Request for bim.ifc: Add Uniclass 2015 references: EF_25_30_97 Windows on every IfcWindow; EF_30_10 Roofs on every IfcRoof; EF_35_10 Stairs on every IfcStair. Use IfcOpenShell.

First a look at what the model holds.

```python
import ifcopenshell

model = ifcopenshell.open("bim.ifc")
print(model.schema)
print("classifications:", [c.Name for c in model.by_type("IfcClassification")])
for ifc_class in ("IfcDoor", "IfcRoof", "IfcStair", "IfcWall", "IfcWindow"):
    print(ifc_class, len(model.by_type(ifc_class)))
```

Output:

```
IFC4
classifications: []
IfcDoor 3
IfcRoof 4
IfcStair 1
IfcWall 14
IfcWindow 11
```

```python
import ifcopenshell
import ifcopenshell.api.classification

model = ifcopenshell.open("bim.ifc")

system = ifcopenshell.api.classification.add_classification(model, classification="Uniclass 2015")

codes = {
    "IfcWindow": ("EF_25_30_97", "Windows"),
    "IfcRoof": ("EF_30_10", "Roofs"),
    "IfcStair": ("EF_35_10", "Stairs"),
}
for ifc_class, (code, name) in codes.items():
    products = model.by_type(ifc_class)
    ifcopenshell.api.classification.add_reference(
        model, products=products, classification=system, identification=code, name=name
    )
    print(code, len(products))

model.write("bim_edited.ifc")
```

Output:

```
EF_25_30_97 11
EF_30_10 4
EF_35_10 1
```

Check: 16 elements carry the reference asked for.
